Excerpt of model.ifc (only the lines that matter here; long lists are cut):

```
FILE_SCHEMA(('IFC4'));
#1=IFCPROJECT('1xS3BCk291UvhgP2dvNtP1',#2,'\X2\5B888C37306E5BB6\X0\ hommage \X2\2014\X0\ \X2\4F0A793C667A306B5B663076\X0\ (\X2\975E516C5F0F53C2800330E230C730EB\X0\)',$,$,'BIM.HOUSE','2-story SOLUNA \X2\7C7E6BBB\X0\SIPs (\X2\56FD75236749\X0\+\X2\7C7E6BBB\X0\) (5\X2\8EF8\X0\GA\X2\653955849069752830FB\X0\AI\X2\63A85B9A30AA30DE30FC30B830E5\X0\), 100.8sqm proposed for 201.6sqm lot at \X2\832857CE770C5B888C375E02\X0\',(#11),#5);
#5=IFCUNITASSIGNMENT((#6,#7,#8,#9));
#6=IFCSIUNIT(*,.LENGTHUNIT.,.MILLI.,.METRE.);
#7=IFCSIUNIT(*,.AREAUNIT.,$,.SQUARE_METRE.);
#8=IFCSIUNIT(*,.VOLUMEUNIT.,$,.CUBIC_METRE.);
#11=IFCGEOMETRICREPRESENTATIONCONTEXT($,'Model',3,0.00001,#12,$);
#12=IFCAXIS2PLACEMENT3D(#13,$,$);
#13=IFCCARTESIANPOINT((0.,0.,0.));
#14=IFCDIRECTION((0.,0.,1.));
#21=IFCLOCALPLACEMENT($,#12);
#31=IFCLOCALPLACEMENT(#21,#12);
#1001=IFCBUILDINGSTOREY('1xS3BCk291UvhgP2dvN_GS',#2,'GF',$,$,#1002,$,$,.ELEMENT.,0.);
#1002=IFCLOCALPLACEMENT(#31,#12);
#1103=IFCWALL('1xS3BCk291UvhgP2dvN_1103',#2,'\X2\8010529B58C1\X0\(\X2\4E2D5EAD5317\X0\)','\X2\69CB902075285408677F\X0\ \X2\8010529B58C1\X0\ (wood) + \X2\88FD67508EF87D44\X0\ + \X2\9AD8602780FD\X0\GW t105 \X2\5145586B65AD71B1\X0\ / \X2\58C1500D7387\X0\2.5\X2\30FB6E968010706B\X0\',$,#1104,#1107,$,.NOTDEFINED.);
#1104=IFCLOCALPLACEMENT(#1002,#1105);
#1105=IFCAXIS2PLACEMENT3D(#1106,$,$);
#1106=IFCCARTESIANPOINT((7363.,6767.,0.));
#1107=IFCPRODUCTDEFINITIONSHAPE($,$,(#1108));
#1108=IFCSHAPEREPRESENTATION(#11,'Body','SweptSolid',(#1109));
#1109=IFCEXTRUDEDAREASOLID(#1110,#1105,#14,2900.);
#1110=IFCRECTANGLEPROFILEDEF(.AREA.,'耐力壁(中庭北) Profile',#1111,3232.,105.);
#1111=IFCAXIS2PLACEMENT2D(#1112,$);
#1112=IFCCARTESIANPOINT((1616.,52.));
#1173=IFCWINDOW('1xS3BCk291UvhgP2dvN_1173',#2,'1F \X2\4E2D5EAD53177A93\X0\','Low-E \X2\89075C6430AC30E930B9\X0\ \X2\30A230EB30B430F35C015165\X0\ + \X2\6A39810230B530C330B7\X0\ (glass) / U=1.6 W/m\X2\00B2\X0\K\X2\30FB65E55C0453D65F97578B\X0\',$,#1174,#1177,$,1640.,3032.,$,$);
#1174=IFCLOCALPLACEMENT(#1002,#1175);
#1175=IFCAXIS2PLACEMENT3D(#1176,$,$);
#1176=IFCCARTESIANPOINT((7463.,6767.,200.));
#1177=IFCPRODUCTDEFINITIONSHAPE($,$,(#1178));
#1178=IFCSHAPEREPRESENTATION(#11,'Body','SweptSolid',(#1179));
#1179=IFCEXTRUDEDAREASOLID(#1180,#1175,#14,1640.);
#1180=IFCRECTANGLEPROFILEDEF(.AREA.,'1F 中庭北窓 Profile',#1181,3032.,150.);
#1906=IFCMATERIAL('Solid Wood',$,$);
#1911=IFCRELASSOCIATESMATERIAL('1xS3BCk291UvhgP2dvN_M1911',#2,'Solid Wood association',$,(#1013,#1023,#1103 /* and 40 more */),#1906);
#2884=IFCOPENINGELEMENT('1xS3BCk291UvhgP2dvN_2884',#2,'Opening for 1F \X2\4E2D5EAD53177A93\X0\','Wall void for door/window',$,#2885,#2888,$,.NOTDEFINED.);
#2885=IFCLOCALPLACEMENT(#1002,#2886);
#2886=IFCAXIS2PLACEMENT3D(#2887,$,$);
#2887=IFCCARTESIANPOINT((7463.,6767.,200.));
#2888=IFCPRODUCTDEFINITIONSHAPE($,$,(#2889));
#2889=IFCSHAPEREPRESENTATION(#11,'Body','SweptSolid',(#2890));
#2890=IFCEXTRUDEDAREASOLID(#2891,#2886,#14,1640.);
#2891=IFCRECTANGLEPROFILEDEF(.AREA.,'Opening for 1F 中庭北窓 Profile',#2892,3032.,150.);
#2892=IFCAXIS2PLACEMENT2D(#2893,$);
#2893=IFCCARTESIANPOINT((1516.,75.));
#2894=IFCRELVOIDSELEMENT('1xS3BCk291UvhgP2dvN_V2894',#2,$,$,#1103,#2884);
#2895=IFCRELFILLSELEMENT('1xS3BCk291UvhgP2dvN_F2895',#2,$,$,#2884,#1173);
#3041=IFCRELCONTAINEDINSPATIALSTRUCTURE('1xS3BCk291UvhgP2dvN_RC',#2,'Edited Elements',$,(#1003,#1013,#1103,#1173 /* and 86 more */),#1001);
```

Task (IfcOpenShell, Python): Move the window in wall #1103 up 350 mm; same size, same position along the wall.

```python
import numpy as np
import ifcopenshell
import ifcopenshell.api.geometry
import ifcopenshell.util.placement
import ifcopenshell.util.unit

model = ifcopenshell.open("model.ifc")
unit_scale = ifcopenshell.util.unit.calculate_unit_scale(model)

window = model.by_guid("1xS3BCk291UvhgP2dvN_1173")
opening = window.FillsVoids[0].RelatingOpeningElement
dz = 0.35 / unit_scale

shift = np.array([0.0, 0.0, dz])
# The window is not placed relative to its opening, so move both.
for product in (opening, window):
    matrix = ifcopenshell.util.placement.get_local_placement(product.ObjectPlacement)
    matrix[:3, 3] += shift
    ifcopenshell.api.geometry.edit_object_placement(model, product=product, matrix=matrix, is_si=False)

print(f"moved by {dz * unit_scale:+.3f} m")

model.write("model_rev.ifc")
```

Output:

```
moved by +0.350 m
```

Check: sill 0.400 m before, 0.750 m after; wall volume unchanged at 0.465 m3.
